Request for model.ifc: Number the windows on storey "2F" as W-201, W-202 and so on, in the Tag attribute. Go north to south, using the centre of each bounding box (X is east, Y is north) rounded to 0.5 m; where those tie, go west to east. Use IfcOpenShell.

First a look at what the model holds.

```python
import ifcopenshell
import ifcopenshell.util.element
import ifcopenshell.util.placement

model = ifcopenshell.open("model.ifc")
print(model.schema)
storey = next(s for s in model.by_type("IfcBuildingStorey") if s.Name == "2F")
windows = [e for e in ifcopenshell.util.element.get_decomposition(storey) if e.is_a("IfcWindow")]
for e in sorted(windows, key=lambda e: e.id()):
    origin = ifcopenshell.util.placement.get_local_placement(e.ObjectPlacement)[:3, 3]
    print(e.id(), e.Tag, e.Name, origin.round(2) + 0.0, sep=" | ")
```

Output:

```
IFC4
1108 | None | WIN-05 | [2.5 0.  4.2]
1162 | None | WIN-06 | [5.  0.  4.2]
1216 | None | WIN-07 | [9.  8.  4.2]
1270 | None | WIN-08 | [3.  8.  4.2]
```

```python
import ifcopenshell
import ifcopenshell.geom
import ifcopenshell.util.element
import ifcopenshell.util.shape

model = ifcopenshell.open("model.ifc")
settings = ifcopenshell.geom.settings()
settings.set("use-world-coords", True)


def centre(element):
    shape = ifcopenshell.geom.create_shape(settings, element)
    return ifcopenshell.util.shape.get_bbox_centroid(shape.geometry)


storey = next(s for s in model.by_type("IfcBuildingStorey") if s.Name == "2F")
windows = [e for e in ifcopenshell.util.element.get_decomposition(storey) if e.is_a("IfcWindow")]

# Insertion points can sit at a corner or the storey origin, so sort by the geometry (in metres).
centres = {e: centre(e) for e in windows}
windows.sort(key=lambda e: (-round(centres[e][1] / 0.5), centres[e][0]))

for i, e in enumerate(windows, start=1):
    number = f"W-2{i:02d}"
    e.Tag = number
    print(e.id(), number)

model.write("model_v2.ifc")
```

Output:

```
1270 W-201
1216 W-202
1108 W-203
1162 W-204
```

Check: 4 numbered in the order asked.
